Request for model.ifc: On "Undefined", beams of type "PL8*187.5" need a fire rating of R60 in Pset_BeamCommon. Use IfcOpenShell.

First a look at what the model holds.

```python
import ifcopenshell
import ifcopenshell.util.element

model = ifcopenshell.open("model.ifc")
print(model.schema)
storey = next(s for s in model.by_type("IfcBuildingStorey") if s.Name == "Undefined")
beams = [e for e in ifcopenshell.util.element.get_decomposition(storey) if e.is_a("IfcBeam")]
seen = {}
for e in beams:
    element_type = ifcopenshell.util.element.get_type(e)
    key = (element_type.Name if element_type != e and element_type else None, ifcopenshell.util.element.get_pset(e, "Pset_BeamCommon", "FireRating"))
    seen[key] = seen.get(key, 0) + 1
for (name, value), count in sorted(seen.items(), key=str):
    print(count, "x", name, "|", value)
```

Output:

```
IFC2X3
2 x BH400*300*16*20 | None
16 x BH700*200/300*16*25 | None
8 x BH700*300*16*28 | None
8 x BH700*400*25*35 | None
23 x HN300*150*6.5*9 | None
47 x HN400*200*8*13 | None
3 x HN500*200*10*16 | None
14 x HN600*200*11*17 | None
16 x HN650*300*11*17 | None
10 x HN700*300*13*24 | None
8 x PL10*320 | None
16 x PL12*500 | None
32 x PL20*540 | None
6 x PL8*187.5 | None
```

```python
import ifcopenshell
import ifcopenshell.api.pset
import ifcopenshell.util.element

model = ifcopenshell.open("model.ifc")

storey = next(s for s in model.by_type("IfcBuildingStorey") if s.Name == "Undefined")
beams = [e for e in ifcopenshell.util.element.get_decomposition(storey) if e.is_a("IfcBeam")]

count = 0
for e in beams:
    element_type = ifcopenshell.util.element.get_type(e)
    if element_type in (None, e) or element_type.Name != "PL8*187.5":
        continue
    # add_pset returns the element's existing set when there is one.
    pset = ifcopenshell.api.pset.add_pset(model, product=e, name="Pset_BeamCommon")
    ifcopenshell.api.pset.edit_pset(model, pset=pset, properties={"FireRating": "R60"})
    count += 1

print(count, "beams updated")

model.write("model_rev.ifc")
```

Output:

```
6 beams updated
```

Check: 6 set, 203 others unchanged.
